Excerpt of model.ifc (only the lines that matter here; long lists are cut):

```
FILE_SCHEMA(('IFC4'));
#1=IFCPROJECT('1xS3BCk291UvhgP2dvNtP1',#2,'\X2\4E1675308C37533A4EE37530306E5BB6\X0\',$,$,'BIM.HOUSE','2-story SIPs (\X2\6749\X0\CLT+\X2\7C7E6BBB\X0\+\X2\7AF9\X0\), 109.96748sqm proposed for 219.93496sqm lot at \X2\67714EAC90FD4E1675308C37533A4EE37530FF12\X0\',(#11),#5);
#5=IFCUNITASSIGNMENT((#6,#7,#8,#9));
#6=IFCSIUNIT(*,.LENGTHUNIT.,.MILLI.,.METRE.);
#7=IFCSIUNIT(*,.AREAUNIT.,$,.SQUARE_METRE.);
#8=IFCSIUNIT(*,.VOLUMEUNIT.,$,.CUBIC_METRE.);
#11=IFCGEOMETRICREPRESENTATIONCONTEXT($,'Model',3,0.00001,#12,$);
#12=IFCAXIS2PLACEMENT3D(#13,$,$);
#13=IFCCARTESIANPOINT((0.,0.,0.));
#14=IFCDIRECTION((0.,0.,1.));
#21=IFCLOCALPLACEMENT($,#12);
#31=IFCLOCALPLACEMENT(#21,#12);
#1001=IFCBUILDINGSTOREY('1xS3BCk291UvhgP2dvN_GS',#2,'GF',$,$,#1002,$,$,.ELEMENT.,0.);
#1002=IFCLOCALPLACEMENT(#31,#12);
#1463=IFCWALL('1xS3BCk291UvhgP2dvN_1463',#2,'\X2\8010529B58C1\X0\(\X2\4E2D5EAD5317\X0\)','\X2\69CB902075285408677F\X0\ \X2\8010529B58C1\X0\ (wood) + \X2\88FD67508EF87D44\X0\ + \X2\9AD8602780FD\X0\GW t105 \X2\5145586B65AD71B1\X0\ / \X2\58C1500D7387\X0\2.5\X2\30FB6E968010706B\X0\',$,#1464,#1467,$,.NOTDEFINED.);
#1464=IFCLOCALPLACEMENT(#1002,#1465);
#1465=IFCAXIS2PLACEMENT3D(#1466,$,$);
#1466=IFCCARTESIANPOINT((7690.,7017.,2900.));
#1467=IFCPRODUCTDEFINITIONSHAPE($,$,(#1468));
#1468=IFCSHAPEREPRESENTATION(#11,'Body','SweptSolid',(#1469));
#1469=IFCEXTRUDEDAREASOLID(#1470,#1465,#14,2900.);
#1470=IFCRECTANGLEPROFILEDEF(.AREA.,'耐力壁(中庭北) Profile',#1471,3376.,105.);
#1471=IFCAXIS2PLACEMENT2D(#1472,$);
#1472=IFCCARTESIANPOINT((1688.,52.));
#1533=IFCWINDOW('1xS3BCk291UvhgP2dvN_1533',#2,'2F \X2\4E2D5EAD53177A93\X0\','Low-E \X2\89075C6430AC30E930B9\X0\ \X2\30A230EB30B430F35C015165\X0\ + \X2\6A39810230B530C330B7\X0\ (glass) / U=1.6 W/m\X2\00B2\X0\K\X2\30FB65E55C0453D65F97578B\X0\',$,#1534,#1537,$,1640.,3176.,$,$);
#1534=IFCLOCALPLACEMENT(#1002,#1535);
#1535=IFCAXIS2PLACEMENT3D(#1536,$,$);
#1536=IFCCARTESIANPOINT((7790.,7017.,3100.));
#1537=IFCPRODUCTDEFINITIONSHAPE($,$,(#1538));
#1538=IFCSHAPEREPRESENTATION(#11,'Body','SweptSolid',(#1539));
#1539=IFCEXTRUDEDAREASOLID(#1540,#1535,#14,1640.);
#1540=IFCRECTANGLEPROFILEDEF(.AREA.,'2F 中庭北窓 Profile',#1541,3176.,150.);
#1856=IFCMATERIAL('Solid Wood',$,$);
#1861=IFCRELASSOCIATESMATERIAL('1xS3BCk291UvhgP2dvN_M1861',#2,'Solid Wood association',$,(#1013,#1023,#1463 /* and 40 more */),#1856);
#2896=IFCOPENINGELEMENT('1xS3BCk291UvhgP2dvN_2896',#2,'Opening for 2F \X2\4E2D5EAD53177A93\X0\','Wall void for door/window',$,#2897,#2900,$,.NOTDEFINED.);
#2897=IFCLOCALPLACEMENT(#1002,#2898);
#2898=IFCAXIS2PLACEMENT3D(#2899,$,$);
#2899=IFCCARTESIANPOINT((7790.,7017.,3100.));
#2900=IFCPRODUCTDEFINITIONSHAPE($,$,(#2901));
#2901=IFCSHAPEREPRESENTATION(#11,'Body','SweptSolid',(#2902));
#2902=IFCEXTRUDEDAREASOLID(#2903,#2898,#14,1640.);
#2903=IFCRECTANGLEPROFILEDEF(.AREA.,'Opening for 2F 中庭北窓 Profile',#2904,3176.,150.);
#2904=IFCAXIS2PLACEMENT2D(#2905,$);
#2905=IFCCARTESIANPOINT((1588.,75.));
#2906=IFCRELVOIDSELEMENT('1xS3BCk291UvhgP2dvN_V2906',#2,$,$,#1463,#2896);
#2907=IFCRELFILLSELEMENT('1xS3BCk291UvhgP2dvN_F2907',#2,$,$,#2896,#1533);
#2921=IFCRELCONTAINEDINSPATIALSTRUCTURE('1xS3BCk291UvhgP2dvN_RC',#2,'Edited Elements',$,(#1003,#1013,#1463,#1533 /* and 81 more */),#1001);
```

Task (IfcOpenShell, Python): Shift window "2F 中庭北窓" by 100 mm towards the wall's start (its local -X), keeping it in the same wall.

```python
import ifcopenshell
import ifcopenshell.api.geometry
import ifcopenshell.util.placement
import ifcopenshell.util.unit

model = ifcopenshell.open("model.ifc")
unit_scale = ifcopenshell.util.unit.calculate_unit_scale(model)

window = model.by_id(1533)
opening = window.FillsVoids[0].RelatingOpeningElement
wall = opening.VoidsElements[0].RelatingBuildingElement

wall_matrix = ifcopenshell.util.placement.get_local_placement(wall.ObjectPlacement)
shift = wall_matrix[:3, 0] * -0.1 / unit_scale
before = ifcopenshell.util.placement.get_local_placement(window.ObjectPlacement)[:3, 3].copy()

# The window is not placed relative to its opening, so move both.
for product in (opening, window):
    matrix = ifcopenshell.util.placement.get_local_placement(product.ObjectPlacement)
    matrix[:3, 3] += shift
    ifcopenshell.api.geometry.edit_object_placement(model, product=product, matrix=matrix, is_si=False)

after = ifcopenshell.util.placement.get_local_placement(window.ObjectPlacement)[:3, 3]
print("window moved by", (after - before).round(3) + 0.0)

model.write("model_edited.ifc")
```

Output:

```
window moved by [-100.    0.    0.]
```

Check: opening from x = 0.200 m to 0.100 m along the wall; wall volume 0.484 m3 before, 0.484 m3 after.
